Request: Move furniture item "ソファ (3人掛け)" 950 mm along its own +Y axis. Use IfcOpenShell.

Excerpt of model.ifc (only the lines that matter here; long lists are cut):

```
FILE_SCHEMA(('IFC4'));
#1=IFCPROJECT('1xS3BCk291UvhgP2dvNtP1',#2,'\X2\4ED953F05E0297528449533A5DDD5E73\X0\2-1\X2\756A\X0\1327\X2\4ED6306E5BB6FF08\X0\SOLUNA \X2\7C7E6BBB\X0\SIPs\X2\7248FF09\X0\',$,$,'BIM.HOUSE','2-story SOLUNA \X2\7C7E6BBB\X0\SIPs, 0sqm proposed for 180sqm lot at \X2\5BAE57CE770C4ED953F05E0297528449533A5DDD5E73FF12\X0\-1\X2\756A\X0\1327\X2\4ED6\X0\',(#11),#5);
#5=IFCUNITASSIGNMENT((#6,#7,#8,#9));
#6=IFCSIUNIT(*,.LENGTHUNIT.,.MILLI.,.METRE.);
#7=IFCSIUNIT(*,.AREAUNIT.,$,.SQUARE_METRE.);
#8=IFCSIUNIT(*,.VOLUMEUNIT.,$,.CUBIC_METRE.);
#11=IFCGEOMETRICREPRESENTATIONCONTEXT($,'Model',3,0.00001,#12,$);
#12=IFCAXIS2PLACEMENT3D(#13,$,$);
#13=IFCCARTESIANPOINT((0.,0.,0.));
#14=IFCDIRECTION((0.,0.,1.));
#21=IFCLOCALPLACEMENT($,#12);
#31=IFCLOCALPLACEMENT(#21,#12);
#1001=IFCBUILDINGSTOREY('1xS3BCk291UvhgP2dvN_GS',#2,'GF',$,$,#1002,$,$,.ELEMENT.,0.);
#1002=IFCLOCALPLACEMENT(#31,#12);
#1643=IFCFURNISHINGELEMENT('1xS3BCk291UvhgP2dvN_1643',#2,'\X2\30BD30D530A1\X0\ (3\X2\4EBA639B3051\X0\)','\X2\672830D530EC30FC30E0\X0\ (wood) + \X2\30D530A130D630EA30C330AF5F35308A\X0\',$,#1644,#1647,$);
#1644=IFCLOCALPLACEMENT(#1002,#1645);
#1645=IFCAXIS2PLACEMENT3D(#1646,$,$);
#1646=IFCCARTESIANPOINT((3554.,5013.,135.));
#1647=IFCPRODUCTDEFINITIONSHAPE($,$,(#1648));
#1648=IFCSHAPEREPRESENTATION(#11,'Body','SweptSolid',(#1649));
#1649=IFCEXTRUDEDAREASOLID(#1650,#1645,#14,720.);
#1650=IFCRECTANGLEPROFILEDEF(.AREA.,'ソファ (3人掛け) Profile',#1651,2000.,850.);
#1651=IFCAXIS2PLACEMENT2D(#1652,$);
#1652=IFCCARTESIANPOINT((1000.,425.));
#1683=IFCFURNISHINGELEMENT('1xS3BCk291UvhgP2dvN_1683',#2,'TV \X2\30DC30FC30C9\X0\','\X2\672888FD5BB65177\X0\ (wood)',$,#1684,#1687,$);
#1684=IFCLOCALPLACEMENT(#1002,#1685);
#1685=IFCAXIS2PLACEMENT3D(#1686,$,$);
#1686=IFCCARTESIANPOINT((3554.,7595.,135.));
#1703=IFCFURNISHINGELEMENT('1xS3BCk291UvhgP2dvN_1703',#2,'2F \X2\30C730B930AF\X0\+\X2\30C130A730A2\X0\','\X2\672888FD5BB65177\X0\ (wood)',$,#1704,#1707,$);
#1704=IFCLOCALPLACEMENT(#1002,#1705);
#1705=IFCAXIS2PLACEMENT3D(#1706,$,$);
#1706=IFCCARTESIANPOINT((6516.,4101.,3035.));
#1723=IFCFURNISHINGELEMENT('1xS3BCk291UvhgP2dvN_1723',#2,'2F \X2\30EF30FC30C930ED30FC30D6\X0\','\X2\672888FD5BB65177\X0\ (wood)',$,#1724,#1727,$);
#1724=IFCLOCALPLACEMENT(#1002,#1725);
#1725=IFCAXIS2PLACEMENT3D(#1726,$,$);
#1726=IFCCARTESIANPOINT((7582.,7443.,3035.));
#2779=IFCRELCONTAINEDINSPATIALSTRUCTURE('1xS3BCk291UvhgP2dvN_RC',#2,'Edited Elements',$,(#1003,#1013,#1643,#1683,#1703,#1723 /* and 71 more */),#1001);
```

```python
import ifcopenshell
import ifcopenshell.api.geometry
import ifcopenshell.util.placement
import ifcopenshell.util.unit

model = ifcopenshell.open("model.ifc")
unit_scale = ifcopenshell.util.unit.calculate_unit_scale(model)

item = model.by_guid("1xS3BCk291UvhgP2dvN_1643")
matrix = ifcopenshell.util.placement.get_local_placement(item.ObjectPlacement)
matrix[:3, 3] += matrix[:3, 1] * 0.95 / unit_scale
ifcopenshell.api.geometry.edit_object_placement(model, product=item, matrix=matrix, is_si=False)

print(ifcopenshell.util.placement.get_local_placement(item.ObjectPlacement).round(3) + 0.0)

model.write("model_rev.ifc")
```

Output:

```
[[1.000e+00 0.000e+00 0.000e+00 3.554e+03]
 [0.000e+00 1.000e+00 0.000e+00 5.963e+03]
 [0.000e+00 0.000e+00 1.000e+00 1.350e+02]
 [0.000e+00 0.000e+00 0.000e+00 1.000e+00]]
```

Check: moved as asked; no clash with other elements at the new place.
